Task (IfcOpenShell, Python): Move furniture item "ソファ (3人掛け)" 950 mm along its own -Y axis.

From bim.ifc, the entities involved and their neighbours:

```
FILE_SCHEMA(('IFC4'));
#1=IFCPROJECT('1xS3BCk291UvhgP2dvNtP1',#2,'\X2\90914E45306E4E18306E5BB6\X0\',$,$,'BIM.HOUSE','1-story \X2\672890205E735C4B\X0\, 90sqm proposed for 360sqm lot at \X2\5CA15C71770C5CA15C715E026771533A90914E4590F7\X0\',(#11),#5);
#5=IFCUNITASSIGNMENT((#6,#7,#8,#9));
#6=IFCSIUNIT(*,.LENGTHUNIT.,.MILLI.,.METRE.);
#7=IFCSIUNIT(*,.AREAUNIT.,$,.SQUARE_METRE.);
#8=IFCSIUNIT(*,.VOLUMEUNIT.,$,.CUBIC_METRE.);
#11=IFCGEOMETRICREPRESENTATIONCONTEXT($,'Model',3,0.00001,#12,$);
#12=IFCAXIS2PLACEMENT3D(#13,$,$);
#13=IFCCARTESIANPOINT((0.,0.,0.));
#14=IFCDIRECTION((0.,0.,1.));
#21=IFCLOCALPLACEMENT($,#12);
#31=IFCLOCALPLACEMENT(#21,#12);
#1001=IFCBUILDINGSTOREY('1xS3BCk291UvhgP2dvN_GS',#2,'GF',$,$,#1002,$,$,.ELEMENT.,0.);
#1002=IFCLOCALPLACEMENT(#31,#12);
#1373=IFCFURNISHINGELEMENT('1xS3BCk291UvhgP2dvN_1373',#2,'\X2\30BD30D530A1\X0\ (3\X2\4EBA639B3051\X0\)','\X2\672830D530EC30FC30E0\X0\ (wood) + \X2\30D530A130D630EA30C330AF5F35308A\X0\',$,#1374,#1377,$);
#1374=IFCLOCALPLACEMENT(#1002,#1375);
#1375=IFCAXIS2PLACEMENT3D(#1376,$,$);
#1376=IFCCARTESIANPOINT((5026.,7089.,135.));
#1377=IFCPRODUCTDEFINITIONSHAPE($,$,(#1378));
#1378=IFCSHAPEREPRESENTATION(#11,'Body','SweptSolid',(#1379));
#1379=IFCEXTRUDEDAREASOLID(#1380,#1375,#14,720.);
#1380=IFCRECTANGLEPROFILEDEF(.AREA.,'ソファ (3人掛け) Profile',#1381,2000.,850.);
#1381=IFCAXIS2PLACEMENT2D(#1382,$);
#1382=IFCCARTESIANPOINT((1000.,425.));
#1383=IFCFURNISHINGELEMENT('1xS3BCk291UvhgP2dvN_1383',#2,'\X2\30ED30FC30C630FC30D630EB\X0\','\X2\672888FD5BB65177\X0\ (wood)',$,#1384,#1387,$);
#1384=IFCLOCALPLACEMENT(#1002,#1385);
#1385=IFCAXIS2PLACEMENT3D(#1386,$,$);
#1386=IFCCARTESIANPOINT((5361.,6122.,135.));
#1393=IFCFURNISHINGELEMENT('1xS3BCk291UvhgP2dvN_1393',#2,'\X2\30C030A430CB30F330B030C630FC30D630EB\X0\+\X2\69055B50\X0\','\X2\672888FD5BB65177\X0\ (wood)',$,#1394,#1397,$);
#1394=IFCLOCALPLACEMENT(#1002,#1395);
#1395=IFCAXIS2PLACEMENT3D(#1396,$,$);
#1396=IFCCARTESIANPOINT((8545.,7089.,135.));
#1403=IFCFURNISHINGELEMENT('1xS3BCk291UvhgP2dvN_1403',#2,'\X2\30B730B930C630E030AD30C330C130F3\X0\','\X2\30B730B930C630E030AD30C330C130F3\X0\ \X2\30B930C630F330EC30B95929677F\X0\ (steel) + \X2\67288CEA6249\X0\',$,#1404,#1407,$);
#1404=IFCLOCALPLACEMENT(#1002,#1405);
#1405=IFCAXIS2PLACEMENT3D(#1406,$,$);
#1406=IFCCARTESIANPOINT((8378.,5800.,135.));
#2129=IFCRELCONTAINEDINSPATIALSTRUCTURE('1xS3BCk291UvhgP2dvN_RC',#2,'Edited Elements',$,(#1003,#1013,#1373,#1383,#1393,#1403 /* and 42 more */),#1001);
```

```python
import ifcopenshell
import ifcopenshell.api.geometry
import ifcopenshell.util.placement
import ifcopenshell.util.unit

model = ifcopenshell.open("bim.ifc")
unit_scale = ifcopenshell.util.unit.calculate_unit_scale(model)

item = model.by_guid("1xS3BCk291UvhgP2dvN_1373")
matrix = ifcopenshell.util.placement.get_local_placement(item.ObjectPlacement)
matrix[:3, 3] -= matrix[:3, 1] * 0.95 / unit_scale
ifcopenshell.api.geometry.edit_object_placement(model, product=item, matrix=matrix, is_si=False)

print(ifcopenshell.util.placement.get_local_placement(item.ObjectPlacement).round(3) + 0.0)

model.write("bim_rev.ifc")
```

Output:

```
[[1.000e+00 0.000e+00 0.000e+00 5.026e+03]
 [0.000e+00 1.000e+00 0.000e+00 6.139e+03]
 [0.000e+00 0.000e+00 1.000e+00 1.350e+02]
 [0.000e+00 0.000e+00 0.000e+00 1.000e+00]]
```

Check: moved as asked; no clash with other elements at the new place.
